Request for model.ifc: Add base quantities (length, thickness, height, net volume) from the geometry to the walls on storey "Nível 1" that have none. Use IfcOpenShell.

First a look at what the model holds.

```python
import ifcopenshell
import ifcopenshell.util.element
import ifcopenshell.util.unit

model = ifcopenshell.open("model.ifc")
print(model.schema)
for unit_type in ("LENGTHUNIT", "AREAUNIT", "VOLUMEUNIT"):
    print(unit_type, ifcopenshell.util.unit.calculate_unit_scale(model, unit_type))
storey = next(s for s in model.by_type("IfcBuildingStorey") if s.Name == "Nível 1")
walls = [e for e in ifcopenshell.util.element.get_decomposition(storey) if e.is_a("IfcWall")]
for e in sorted(walls, key=lambda e: e.id()):
    print(e.id(), e.is_a(), e.Name, list(ifcopenshell.util.element.get_psets(e, qtos_only=True)), sep=" | ")
```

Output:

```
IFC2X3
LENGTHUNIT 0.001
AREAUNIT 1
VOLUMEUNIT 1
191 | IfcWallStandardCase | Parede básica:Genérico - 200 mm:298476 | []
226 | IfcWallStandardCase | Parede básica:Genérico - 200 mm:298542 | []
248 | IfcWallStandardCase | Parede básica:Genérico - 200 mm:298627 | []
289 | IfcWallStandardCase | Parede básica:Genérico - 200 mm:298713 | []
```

```python
import ifcopenshell
import ifcopenshell.api.pset
import ifcopenshell.geom
import ifcopenshell.util.element
import ifcopenshell.util.shape
import ifcopenshell.util.unit

model = ifcopenshell.open("model.ifc")
unit_scale = ifcopenshell.util.unit.calculate_unit_scale(model)
volume_scale = ifcopenshell.util.unit.calculate_unit_scale(model, "VOLUMEUNIT")
settings = ifcopenshell.geom.settings()

storey = next(s for s in model.by_type("IfcBuildingStorey") if s.Name == "Nível 1")
walls = [e for e in ifcopenshell.util.element.get_decomposition(storey) if e.is_a("IfcWall")]

for e in sorted(walls, key=lambda e: e.id()):
    if ifcopenshell.util.element.get_psets(e, qtos_only=True, should_inherit=False):
        continue
    # Geometry comes back in metres, in the element's own axes.
    shape = ifcopenshell.geom.create_shape(settings, e)
    values = {
        "Length": ifcopenshell.util.shape.get_x(shape.geometry) / unit_scale,
        "Width": ifcopenshell.util.shape.get_y(shape.geometry) / unit_scale,
        "Height": ifcopenshell.util.shape.get_z(shape.geometry) / unit_scale,
        "NetVolume": ifcopenshell.util.shape.get_volume(shape.geometry) / volume_scale,
    }
    qto = ifcopenshell.api.pset.add_qto(model, product=e, name="BaseQuantities")
    ifcopenshell.api.pset.edit_qto(model, qto=qto, properties=values)
    print(e.id(), {k: round(v, 3) for k, v in values.items()})

model.write("model_updated.ifc")
```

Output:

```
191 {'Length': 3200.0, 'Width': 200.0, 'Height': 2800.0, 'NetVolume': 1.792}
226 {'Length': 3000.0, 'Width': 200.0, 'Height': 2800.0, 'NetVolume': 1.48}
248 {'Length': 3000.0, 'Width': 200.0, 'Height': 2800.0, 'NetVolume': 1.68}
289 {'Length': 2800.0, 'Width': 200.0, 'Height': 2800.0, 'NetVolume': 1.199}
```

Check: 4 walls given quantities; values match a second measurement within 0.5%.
